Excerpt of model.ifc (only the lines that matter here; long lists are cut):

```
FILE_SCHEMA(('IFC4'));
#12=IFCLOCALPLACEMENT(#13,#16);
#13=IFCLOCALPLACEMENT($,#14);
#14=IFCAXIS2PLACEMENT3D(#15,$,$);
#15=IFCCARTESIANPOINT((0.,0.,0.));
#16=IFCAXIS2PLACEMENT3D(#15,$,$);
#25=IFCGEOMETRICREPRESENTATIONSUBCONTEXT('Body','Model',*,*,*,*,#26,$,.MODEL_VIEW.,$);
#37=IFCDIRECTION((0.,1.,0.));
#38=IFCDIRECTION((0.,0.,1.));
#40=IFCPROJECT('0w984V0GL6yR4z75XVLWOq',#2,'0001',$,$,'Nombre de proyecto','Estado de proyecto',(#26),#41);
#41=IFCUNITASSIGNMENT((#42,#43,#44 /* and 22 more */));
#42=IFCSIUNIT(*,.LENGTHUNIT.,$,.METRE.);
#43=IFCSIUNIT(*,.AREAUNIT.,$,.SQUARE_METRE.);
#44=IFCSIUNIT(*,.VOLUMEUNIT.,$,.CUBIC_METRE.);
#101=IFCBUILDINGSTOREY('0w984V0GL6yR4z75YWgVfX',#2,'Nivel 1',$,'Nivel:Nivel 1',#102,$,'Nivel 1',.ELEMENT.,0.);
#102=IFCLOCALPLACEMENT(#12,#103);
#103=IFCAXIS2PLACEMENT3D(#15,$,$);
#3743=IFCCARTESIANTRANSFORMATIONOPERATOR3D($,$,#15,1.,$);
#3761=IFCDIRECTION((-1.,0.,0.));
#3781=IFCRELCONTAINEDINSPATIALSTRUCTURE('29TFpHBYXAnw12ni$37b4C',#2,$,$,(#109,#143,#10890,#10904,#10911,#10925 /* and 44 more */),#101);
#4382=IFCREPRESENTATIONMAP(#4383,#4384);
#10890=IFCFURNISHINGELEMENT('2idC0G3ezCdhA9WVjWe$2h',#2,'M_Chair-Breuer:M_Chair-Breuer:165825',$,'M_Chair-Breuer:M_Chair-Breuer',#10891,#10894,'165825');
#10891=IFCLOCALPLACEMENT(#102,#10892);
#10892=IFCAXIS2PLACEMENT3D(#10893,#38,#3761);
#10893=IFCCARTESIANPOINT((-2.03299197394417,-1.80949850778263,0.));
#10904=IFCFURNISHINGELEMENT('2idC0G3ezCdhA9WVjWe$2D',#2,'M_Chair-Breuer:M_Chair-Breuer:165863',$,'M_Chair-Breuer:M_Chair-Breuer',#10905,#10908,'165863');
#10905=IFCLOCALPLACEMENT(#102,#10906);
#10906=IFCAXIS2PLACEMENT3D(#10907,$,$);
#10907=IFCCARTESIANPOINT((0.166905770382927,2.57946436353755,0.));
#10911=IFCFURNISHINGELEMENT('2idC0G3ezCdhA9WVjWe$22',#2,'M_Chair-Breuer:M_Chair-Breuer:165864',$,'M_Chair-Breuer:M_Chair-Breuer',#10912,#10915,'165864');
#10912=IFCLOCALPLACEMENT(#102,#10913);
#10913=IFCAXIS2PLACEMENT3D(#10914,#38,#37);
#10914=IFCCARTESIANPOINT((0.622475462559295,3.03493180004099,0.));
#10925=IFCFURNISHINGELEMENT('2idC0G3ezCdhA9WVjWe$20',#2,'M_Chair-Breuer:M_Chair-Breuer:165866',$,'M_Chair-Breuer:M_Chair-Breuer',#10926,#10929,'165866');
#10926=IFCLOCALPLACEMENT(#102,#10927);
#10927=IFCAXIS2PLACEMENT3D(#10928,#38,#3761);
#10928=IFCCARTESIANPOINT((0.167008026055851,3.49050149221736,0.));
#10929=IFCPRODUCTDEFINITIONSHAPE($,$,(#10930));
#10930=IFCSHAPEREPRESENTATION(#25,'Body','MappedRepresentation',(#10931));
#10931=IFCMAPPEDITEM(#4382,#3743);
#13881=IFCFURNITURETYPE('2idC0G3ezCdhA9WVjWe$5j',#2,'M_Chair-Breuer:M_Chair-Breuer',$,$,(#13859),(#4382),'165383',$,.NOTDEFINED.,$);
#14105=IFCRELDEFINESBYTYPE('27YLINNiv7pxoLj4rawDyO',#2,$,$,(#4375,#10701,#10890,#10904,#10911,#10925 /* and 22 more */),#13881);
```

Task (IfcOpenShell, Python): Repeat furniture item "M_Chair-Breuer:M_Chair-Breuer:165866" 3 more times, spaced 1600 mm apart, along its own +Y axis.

```python
import ifcopenshell
import ifcopenshell.api.geometry
import ifcopenshell.api.root
import ifcopenshell.util.element
import ifcopenshell.util.placement

model = ifcopenshell.open("model.ifc")


def reuse_history(source, copy):
    """copy_class also copies each property set's owner history, people and application; keep the originals."""
    for rel in copy.IsDefinedBy:
        if rel.is_a("IfcRelDefinesByProperties") and (history := rel.RelatingPropertyDefinition.OwnerHistory):
            rel.RelatingPropertyDefinition.OwnerHistory = source.OwnerHistory
            ifcopenshell.util.element.remove_deep2(model, history)


source = model.by_id(10925)
base = ifcopenshell.util.placement.get_local_placement(source.ObjectPlacement)
step = base[:3, 1] * 1.6

for i in range(1, 4):
    copy = ifcopenshell.api.root.copy_class(model, product=source)
    copy.Representation = ifcopenshell.util.element.copy_deep(
        model, source.Representation, exclude=["IfcGeometricRepresentationContext", "IfcRepresentationMap"]
    )
    copy.Name = "M_Chair-Breuer:M_Chair-Breuer"
    copy.Tag = None
    reuse_history(source, copy)
    matrix = base.copy()
    matrix[:3, 3] += i * step
    print("added at", matrix[:3, 3].round(3) + 0.0)
    ifcopenshell.api.geometry.edit_object_placement(model, product=copy, matrix=matrix, is_si=False)

model.write("model_updated.ifc")
```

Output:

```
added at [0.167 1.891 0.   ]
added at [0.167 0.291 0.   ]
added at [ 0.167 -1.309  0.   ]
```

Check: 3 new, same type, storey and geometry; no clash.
